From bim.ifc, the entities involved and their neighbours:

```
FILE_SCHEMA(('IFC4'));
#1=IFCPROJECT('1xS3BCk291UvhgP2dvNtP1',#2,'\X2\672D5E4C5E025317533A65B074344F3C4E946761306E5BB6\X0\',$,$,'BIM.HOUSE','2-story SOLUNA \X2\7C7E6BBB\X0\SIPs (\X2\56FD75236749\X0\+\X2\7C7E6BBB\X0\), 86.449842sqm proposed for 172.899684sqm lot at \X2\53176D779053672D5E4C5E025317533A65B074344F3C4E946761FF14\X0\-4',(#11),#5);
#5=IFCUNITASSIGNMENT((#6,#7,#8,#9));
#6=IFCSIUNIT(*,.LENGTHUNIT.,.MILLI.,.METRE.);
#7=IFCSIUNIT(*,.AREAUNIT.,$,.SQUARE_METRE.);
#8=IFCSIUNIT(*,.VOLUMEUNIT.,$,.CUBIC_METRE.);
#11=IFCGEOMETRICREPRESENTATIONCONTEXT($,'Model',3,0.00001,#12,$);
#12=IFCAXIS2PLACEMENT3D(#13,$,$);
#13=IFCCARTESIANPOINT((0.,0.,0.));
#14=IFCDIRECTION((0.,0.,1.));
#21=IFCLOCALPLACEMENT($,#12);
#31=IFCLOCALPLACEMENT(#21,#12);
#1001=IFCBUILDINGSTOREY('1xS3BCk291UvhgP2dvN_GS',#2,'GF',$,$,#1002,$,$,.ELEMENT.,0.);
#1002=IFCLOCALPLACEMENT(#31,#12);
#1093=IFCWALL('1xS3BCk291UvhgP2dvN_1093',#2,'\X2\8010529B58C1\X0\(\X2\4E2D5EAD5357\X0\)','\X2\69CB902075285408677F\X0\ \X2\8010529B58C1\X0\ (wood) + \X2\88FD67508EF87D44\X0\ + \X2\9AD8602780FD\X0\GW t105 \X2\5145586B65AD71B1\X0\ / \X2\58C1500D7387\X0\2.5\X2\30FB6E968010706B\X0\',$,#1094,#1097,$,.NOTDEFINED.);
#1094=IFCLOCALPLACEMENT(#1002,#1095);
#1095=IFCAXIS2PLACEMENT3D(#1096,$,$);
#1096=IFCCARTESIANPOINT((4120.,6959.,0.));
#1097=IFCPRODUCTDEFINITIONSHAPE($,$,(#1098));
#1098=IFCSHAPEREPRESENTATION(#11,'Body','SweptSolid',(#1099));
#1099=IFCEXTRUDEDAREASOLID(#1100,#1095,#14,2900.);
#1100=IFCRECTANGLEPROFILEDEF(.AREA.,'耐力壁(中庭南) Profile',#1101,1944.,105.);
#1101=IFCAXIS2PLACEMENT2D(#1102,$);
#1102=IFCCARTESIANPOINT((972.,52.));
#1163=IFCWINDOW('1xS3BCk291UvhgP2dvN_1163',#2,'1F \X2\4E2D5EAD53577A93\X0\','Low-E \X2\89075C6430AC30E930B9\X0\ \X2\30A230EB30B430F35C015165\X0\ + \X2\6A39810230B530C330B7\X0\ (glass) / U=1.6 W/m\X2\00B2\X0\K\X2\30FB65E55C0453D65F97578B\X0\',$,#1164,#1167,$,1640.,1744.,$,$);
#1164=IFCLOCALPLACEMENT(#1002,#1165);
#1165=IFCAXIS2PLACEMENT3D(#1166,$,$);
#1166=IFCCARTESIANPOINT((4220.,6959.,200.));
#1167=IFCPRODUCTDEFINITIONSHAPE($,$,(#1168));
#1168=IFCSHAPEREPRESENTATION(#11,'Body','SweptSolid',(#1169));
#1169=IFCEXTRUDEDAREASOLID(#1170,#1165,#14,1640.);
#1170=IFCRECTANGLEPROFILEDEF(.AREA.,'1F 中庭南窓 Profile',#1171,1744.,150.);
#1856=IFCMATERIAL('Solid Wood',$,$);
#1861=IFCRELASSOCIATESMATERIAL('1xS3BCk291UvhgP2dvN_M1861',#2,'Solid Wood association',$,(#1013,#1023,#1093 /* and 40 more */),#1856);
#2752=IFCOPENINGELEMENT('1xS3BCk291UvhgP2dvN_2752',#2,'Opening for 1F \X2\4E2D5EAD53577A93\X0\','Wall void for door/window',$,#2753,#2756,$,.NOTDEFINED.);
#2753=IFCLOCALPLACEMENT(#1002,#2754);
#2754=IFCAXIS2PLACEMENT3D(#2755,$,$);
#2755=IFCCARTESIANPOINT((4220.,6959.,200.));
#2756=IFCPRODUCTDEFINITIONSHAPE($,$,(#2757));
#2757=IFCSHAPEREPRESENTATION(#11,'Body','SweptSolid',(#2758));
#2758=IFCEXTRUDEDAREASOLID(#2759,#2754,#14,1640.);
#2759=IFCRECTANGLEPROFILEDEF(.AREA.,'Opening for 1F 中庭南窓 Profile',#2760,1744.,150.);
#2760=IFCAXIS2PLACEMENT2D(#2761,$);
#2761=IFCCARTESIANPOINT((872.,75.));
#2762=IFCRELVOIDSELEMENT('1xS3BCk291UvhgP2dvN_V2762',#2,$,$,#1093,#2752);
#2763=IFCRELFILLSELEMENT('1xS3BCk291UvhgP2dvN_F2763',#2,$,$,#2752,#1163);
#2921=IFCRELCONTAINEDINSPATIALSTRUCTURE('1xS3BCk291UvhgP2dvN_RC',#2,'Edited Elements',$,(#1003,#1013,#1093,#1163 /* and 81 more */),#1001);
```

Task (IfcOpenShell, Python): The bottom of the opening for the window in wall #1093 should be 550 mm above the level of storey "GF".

```python
import numpy as np
import ifcopenshell
import ifcopenshell.api.geometry
import ifcopenshell.geom
import ifcopenshell.util.element
import ifcopenshell.util.placement
import ifcopenshell.util.shape
import ifcopenshell.util.unit

model = ifcopenshell.open("bim.ifc")
unit_scale = ifcopenshell.util.unit.calculate_unit_scale(model)

window = model.by_id(1163)
opening = window.FillsVoids[0].RelatingOpeningElement
storey = ifcopenshell.util.element.get_container(window, ifc_class="IfcBuildingStorey")
level = ifcopenshell.util.placement.get_local_placement(storey.ObjectPlacement)[2, 3]

# The opening's origin need not be at the sill, so measure its lowest point.
shape = ifcopenshell.geom.create_shape(ifcopenshell.geom.settings(), opening)
bottom = ifcopenshell.util.shape.get_shape_bottom_elevation(shape, shape.geometry) / unit_scale
dz = level + 550.0 - bottom

shift = np.array([0.0, 0.0, dz])
# The window is not placed relative to its opening, so move both.
for product in (opening, window):
    matrix = ifcopenshell.util.placement.get_local_placement(product.ObjectPlacement)
    matrix[:3, 3] += shift
    ifcopenshell.api.geometry.edit_object_placement(model, product=product, matrix=matrix, is_si=False)

print(f"moved by {dz * unit_scale:+.3f} m")

model.write("bim_v2.ifc")
```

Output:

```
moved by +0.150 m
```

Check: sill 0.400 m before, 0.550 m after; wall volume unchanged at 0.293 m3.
